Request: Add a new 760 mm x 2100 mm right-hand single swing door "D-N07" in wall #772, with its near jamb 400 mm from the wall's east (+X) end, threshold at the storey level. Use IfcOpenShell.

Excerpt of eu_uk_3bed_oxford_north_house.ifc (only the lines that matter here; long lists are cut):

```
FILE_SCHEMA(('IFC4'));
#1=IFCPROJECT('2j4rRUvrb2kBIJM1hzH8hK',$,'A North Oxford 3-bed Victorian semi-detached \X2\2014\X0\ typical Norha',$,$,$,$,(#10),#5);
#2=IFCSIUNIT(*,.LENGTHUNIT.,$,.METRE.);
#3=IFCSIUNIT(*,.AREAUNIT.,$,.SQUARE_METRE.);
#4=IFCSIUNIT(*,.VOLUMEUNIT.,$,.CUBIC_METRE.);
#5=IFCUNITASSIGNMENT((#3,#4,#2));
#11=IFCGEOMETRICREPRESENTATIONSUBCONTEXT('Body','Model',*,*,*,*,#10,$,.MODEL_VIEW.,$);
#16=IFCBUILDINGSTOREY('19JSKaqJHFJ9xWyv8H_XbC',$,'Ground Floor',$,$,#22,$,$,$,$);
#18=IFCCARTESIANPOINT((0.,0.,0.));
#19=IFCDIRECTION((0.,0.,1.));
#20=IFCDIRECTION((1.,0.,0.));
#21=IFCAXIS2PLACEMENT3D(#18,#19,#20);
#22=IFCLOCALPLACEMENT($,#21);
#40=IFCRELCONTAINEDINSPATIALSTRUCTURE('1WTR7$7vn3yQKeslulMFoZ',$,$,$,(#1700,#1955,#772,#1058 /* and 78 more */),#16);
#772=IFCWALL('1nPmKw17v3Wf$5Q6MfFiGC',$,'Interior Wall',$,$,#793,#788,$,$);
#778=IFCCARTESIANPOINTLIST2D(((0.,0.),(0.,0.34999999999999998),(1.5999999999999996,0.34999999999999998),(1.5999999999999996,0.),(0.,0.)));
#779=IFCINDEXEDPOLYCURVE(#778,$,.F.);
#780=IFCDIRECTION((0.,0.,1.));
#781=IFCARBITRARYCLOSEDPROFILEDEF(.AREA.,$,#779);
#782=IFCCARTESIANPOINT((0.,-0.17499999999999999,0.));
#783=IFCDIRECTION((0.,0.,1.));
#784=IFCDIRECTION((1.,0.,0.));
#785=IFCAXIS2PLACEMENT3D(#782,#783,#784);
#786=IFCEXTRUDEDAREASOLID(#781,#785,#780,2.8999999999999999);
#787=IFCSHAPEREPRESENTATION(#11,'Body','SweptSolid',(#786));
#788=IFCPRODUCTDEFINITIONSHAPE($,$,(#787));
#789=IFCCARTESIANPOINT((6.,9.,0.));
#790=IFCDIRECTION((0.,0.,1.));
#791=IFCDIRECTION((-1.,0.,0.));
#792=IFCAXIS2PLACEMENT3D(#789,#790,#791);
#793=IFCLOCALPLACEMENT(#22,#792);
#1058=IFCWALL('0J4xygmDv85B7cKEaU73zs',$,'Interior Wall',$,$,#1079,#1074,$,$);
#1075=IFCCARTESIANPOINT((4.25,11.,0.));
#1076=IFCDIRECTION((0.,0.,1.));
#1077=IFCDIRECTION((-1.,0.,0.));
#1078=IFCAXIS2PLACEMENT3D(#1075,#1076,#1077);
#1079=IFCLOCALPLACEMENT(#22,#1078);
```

```python
import numpy as np
import ifcopenshell
import ifcopenshell.api.feature
import ifcopenshell.api.geometry
import ifcopenshell.api.root
import ifcopenshell.api.spatial
import ifcopenshell.geom
import ifcopenshell.util.element
import ifcopenshell.util.placement
import ifcopenshell.util.representation
import ifcopenshell.util.shape
import ifcopenshell.util.unit

model = ifcopenshell.open("eu_uk_3bed_oxford_north_house.ifc")
unit_scale = ifcopenshell.util.unit.calculate_unit_scale(model)
settings = ifcopenshell.geom.settings()


def volume(element):
    """Net volume in cubic metres, openings subtracted."""
    shape = ifcopenshell.geom.create_shape(settings, element)
    return ifcopenshell.util.shape.get_volume(shape.geometry)


wall = model.by_id(772)
storey = ifcopenshell.util.element.get_container(wall, ifc_class="IfcBuildingStorey")
context = ifcopenshell.util.representation.get_context(model, "Model", "Body", "MODEL_VIEW")
before = volume(wall)

width, height, from_end, sill = 0.76, 2.1, 0.4, 0.0  # metres

# The wall runs along its own X axis, and the end named is its -X end.
wall_shape = ifcopenshell.geom.create_shape(settings, wall)
x, y, z = ifcopenshell.util.shape.get_vertices(wall_shape.geometry).T
start = x.min() + from_end
face, thickness = float(y.min()), float(y.max() - y.min())
wall_matrix = ifcopenshell.util.placement.get_local_placement(wall.ObjectPlacement)
level = ifcopenshell.util.placement.get_local_placement(storey.ObjectPlacement)[2, 3]


def in_wall(x, y):
    """Placement at x, y metres in the wall's axes, at sill height."""
    matrix = wall_matrix.copy()
    matrix[:, 3] = wall_matrix @ np.array([x / unit_scale, y / unit_scale, 0.0, 1.0])
    matrix[2, 3] = level + sill / unit_scale
    return matrix


# Opening: a box that overshoots both wall faces by 50 mm.
opening = ifcopenshell.api.root.create_entity(model, ifc_class="IfcOpeningElement", predefined_type="OPENING")
box = ifcopenshell.api.geometry.add_wall_representation(
    model, context=context, length=width, height=height, thickness=thickness + 0.1
)
ifcopenshell.api.geometry.assign_representation(model, product=opening, representation=box)
ifcopenshell.api.geometry.edit_object_placement(model, product=opening, matrix=in_wall(start, face - 0.05), is_si=False)
ifcopenshell.api.feature.add_feature(model, feature=opening, element=wall)

door = ifcopenshell.api.root.create_entity(model, ifc_class="IfcDoor", name="D-N07", predefined_type="DOOR")
door.OverallWidth, door.OverallHeight = width / unit_scale, height / unit_scale
door.OperationType = "SINGLE_SWING_RIGHT"
body = ifcopenshell.api.geometry.add_door_representation(
    model,
    context=context,
    overall_width=door.OverallWidth,
    overall_height=door.OverallHeight,
    operation_type="SINGLE_SWING_RIGHT",
    lining_properties={"LiningDepth": thickness / unit_scale, "ThresholdDepth": thickness / unit_scale},
)
ifcopenshell.api.geometry.assign_representation(model, product=door, representation=body)
ifcopenshell.api.spatial.assign_container(model, products=[door], relating_structure=storey)
ifcopenshell.api.feature.add_filling(model, opening=opening, element=door)

# The lining spans the wall, so the door starts at the wall face.
ifcopenshell.api.geometry.edit_object_placement(model, product=door, matrix=in_wall(start, face), is_si=False)

after = volume(wall)

print(f"wall volume {before:.3f} -> {after:.3f} m3")

model.write("eu_uk_3bed_oxford_north_house-out.ifc")
```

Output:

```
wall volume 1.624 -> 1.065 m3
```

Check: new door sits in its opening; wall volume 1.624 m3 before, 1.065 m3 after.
